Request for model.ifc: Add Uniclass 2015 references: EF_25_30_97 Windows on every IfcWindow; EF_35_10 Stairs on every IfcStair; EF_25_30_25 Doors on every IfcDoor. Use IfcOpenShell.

First a look at what the model holds.

```python
import ifcopenshell

model = ifcopenshell.open("model.ifc")
print(model.schema)
print("classifications:", [c.Name for c in model.by_type("IfcClassification")])
for ifc_class in ("IfcDoor", "IfcRoof", "IfcStair", "IfcWall", "IfcWindow"):
    print(ifc_class, len(model.by_type(ifc_class)))
```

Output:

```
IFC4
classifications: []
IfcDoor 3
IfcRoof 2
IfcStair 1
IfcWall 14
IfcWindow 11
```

```python
import ifcopenshell
import ifcopenshell.api.classification

model = ifcopenshell.open("model.ifc")

system = ifcopenshell.api.classification.add_classification(model, classification="Uniclass 2015")

codes = {
    "IfcWindow": ("EF_25_30_97", "Windows"),
    "IfcStair": ("EF_35_10", "Stairs"),
    "IfcDoor": ("EF_25_30_25", "Doors"),
}
for ifc_class, (code, name) in codes.items():
    products = model.by_type(ifc_class)
    ifcopenshell.api.classification.add_reference(
        model, products=products, classification=system, identification=code, name=name
    )
    print(code, len(products))

model.write("model_v2.ifc")
```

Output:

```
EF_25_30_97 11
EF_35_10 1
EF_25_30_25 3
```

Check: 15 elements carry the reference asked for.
